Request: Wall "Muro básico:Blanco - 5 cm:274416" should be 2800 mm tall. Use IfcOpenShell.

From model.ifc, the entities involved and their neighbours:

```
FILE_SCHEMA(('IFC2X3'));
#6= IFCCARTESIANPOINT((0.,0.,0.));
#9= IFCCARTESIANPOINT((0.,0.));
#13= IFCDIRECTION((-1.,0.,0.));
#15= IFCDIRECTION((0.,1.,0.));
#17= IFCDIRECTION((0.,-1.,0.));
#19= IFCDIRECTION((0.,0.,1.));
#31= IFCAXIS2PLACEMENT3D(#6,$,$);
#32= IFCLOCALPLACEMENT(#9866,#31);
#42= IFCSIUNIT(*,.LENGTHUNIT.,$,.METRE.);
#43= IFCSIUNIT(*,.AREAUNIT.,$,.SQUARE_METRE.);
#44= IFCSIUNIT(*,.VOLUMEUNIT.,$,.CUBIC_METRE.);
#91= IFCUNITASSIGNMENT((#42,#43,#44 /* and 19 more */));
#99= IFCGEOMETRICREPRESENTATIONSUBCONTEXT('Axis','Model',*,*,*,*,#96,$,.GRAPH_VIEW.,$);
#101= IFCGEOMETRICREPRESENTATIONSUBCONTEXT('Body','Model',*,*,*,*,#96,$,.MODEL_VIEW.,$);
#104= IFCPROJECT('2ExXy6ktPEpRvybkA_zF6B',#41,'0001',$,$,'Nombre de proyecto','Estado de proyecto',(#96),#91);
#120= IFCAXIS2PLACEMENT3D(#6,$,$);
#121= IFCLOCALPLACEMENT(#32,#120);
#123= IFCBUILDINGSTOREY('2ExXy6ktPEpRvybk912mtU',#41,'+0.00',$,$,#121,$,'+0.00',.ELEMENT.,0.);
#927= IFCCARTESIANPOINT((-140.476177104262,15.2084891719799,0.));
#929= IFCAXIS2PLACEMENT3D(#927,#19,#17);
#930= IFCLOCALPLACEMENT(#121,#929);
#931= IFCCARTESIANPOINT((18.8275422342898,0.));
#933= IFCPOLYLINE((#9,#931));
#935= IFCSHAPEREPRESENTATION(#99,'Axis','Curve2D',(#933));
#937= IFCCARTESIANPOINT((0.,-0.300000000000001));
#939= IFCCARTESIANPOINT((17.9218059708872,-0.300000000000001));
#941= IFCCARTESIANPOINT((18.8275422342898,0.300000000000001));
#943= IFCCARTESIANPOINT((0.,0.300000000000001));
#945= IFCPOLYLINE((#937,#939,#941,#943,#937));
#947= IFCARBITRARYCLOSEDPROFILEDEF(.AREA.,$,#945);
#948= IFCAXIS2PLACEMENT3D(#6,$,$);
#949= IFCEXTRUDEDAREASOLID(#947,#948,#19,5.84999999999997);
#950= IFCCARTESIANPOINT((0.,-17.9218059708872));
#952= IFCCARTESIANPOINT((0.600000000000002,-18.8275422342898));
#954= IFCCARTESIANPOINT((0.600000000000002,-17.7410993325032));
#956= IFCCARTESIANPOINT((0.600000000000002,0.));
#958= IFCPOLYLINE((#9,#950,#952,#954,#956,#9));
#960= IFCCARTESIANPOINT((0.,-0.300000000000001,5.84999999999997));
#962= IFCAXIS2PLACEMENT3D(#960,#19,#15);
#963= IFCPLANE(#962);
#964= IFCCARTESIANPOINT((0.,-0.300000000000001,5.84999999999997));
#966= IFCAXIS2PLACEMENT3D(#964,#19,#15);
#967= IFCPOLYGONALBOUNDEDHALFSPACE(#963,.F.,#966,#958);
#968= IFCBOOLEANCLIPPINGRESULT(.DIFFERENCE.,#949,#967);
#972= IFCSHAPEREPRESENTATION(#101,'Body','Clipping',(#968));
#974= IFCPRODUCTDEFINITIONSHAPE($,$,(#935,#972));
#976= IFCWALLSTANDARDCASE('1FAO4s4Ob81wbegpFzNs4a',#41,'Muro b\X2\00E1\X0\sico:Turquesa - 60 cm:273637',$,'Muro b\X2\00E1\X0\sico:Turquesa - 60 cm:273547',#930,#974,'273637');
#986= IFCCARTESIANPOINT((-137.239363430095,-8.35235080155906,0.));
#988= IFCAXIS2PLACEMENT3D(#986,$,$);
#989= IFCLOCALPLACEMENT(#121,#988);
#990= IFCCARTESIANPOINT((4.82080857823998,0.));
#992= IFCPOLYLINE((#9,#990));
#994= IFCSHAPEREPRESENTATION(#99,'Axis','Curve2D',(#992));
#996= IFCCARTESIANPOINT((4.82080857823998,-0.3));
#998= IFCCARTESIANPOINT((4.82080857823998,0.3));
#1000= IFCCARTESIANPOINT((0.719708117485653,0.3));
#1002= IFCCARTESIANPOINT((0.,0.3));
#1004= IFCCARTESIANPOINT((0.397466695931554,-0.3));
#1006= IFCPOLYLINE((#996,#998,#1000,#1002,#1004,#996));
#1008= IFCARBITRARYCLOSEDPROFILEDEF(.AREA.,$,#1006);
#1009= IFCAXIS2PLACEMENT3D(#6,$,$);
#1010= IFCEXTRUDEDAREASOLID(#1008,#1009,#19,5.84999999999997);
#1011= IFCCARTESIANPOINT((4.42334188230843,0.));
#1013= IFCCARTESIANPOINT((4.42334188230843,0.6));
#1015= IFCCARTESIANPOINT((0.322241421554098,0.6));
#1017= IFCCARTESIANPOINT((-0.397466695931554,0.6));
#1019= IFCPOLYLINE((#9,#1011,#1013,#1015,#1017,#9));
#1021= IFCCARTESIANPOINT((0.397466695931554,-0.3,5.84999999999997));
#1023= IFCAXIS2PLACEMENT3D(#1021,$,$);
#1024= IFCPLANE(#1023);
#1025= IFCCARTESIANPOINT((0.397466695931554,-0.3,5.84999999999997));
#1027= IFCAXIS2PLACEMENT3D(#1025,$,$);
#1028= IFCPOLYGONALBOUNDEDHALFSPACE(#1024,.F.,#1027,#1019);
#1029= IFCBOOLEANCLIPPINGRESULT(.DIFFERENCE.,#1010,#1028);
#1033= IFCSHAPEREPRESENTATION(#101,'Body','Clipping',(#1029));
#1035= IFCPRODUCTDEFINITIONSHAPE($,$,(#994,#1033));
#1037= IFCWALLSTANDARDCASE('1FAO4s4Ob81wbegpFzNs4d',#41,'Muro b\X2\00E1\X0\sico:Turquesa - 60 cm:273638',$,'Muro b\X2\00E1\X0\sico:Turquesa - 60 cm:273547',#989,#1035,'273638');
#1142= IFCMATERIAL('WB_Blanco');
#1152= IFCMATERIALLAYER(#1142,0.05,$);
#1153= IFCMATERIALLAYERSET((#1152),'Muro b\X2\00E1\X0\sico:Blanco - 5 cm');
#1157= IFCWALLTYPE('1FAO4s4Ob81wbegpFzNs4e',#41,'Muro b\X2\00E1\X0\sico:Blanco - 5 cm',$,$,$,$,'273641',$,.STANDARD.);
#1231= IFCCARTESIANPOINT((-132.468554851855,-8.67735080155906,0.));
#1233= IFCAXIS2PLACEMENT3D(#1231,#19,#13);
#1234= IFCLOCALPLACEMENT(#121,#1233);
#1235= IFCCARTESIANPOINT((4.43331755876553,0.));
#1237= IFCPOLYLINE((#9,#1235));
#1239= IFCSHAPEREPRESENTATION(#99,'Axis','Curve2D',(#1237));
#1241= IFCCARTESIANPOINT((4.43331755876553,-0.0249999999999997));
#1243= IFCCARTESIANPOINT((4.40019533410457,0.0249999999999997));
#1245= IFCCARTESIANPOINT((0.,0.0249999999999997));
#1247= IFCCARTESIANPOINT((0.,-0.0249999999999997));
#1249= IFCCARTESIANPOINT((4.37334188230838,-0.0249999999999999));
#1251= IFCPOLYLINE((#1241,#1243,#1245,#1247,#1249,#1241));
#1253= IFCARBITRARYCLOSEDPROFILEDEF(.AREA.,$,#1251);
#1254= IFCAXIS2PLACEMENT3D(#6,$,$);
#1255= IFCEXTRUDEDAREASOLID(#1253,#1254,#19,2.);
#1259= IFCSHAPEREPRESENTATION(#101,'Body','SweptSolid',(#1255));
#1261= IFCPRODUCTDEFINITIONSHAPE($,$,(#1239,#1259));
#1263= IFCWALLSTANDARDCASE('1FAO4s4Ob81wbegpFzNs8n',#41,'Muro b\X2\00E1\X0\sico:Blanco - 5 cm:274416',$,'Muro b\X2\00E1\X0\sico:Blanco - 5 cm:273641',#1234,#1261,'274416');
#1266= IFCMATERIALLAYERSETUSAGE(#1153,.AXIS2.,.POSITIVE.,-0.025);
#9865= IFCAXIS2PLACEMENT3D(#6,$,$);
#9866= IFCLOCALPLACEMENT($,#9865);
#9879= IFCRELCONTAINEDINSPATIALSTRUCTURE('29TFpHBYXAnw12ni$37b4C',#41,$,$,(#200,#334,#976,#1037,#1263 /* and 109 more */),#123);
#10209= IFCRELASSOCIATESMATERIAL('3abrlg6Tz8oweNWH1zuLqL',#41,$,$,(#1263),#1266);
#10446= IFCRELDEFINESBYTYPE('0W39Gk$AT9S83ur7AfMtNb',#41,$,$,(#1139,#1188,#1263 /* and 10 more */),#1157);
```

```python
import ifcopenshell
import ifcopenshell.geom
import ifcopenshell.util.representation
import ifcopenshell.util.shape
import ifcopenshell.util.unit

model = ifcopenshell.open("model.ifc")
unit_scale = ifcopenshell.util.unit.calculate_unit_scale(model)
settings = ifcopenshell.geom.settings()


def volume(element):
    """Net volume in cubic metres, openings subtracted."""
    shape = ifcopenshell.geom.create_shape(settings, element)
    return ifcopenshell.util.shape.get_volume(shape.geometry)


wall = model.by_guid("1FAO4s4Ob81wbegpFzNs8n")
before = volume(wall)

body = ifcopenshell.util.representation.get_representation(wall, "Model", "Body")
solid = body.Items[0]
old_height = solid.Depth
solid.Depth = 2.8 / unit_scale
after = volume(wall)

print(f"height {old_height:g} -> {solid.Depth:g}, volume {before:.3f} -> {after:.3f} m3")

model.write("model_rev.ifc")
```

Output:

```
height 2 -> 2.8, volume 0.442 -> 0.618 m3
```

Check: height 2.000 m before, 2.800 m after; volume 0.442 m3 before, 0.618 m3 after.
